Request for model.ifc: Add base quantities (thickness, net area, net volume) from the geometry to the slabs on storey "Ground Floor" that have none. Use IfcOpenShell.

First a look at what the model holds.

```python
import ifcopenshell
import ifcopenshell.util.element
import ifcopenshell.util.unit

model = ifcopenshell.open("model.ifc")
print(model.schema)
for unit_type in ("LENGTHUNIT", "AREAUNIT", "VOLUMEUNIT"):
    print(unit_type, ifcopenshell.util.unit.calculate_unit_scale(model, unit_type))
storey = next(s for s in model.by_type("IfcBuildingStorey") if s.Name == "Ground Floor")
slabs = [e for e in ifcopenshell.util.element.get_decomposition(storey) if e.is_a("IfcSlab")]
for e in sorted(slabs, key=lambda e: e.id()):
    print(e.id(), e.is_a(), e.Name, list(ifcopenshell.util.element.get_psets(e, qtos_only=True)), sep=" | ")
```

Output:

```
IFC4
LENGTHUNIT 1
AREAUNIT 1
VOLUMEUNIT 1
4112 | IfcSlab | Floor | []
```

```python
import ifcopenshell
import ifcopenshell.api.pset
import ifcopenshell.geom
import ifcopenshell.util.element
import ifcopenshell.util.shape
import ifcopenshell.util.unit

model = ifcopenshell.open("model.ifc")
unit_scale = ifcopenshell.util.unit.calculate_unit_scale(model)
area_scale = ifcopenshell.util.unit.calculate_unit_scale(model, "AREAUNIT")
volume_scale = ifcopenshell.util.unit.calculate_unit_scale(model, "VOLUMEUNIT")
settings = ifcopenshell.geom.settings()

storey = next(s for s in model.by_type("IfcBuildingStorey") if s.Name == "Ground Floor")
slabs = [e for e in ifcopenshell.util.element.get_decomposition(storey) if e.is_a("IfcSlab")]

for e in sorted(slabs, key=lambda e: e.id()):
    if ifcopenshell.util.element.get_psets(e, qtos_only=True, should_inherit=False):
        continue
    # Geometry comes back in metres, in the element's own axes.
    shape = ifcopenshell.geom.create_shape(settings, e)
    values = {
        "Width": ifcopenshell.util.shape.get_z(shape.geometry) / unit_scale,
        "NetArea": ifcopenshell.util.shape.get_footprint_area(shape.geometry) / area_scale,
        "NetVolume": ifcopenshell.util.shape.get_volume(shape.geometry) / volume_scale,
    }
    qto = ifcopenshell.api.pset.add_qto(model, product=e, name="Qto_SlabBaseQuantities")
    ifcopenshell.api.pset.edit_qto(model, qto=qto, properties=values)
    print(e.id(), {k: round(v, 3) for k, v in values.items()})

model.write("model-out.ifc")
```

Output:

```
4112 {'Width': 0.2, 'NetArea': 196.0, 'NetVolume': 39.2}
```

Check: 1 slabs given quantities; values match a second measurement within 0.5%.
